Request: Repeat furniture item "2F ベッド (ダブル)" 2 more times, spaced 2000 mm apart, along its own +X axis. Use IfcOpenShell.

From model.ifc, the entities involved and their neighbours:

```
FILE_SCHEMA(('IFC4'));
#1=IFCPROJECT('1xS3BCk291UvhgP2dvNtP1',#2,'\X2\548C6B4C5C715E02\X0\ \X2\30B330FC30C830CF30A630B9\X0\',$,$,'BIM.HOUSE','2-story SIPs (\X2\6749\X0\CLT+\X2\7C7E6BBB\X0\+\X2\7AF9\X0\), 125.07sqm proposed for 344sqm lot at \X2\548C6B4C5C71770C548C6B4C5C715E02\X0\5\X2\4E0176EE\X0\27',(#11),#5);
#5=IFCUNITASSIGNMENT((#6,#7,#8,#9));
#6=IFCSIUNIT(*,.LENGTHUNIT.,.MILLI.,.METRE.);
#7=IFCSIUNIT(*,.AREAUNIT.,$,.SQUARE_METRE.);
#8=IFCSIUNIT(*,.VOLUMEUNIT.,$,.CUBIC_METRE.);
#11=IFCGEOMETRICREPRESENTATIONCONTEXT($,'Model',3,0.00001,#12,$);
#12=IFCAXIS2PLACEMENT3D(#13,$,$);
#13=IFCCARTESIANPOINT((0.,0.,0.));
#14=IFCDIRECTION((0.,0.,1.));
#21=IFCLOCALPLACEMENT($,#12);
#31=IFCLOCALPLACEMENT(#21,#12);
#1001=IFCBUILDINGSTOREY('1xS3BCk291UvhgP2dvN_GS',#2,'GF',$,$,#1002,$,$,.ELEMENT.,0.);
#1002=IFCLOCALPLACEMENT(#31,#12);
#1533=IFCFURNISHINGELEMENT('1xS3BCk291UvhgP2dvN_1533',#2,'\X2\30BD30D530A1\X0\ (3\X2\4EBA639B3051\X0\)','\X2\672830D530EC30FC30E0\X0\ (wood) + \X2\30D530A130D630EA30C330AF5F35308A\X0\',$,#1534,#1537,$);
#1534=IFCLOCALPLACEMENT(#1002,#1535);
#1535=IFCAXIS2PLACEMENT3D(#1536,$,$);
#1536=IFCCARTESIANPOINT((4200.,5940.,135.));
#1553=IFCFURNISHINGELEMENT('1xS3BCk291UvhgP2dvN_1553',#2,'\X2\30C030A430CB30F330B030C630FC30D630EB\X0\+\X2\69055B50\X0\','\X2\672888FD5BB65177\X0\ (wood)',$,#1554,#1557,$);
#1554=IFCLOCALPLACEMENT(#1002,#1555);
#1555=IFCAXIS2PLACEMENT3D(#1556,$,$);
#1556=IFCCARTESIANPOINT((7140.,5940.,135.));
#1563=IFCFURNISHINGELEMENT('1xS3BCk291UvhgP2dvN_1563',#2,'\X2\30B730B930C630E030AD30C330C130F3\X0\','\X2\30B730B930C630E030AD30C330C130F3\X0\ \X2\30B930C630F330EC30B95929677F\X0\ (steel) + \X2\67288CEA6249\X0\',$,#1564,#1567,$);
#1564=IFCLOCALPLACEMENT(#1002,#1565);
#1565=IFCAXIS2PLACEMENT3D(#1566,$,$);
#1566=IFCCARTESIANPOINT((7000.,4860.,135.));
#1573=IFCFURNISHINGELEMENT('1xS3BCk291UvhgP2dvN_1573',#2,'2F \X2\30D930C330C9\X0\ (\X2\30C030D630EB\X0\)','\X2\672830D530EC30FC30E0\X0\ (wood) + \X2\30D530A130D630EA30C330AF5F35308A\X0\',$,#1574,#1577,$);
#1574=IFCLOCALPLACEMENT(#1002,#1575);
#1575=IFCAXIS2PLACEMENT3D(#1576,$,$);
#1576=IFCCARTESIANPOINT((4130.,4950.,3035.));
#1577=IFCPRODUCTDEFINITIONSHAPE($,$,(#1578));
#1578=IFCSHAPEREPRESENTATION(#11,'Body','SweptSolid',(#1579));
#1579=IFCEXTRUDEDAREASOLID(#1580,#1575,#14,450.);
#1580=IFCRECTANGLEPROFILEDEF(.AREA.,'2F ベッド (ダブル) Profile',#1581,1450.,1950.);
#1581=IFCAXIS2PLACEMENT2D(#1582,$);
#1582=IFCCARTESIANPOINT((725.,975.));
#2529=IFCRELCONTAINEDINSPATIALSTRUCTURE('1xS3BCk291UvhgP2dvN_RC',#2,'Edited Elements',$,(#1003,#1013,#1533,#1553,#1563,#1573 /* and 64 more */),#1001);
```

```python
import ifcopenshell
import ifcopenshell.api.geometry
import ifcopenshell.api.root
import ifcopenshell.util.element
import ifcopenshell.util.placement

model = ifcopenshell.open("model.ifc")


def reuse_history(source, copy):
    """copy_class also copies each property set's owner history, people and application; keep the originals."""
    for rel in copy.IsDefinedBy:
        if rel.is_a("IfcRelDefinesByProperties") and (history := rel.RelatingPropertyDefinition.OwnerHistory):
            rel.RelatingPropertyDefinition.OwnerHistory = source.OwnerHistory
            ifcopenshell.util.element.remove_deep2(model, history)


source = model.by_guid("1xS3BCk291UvhgP2dvN_1573")
base = ifcopenshell.util.placement.get_local_placement(source.ObjectPlacement)
step = base[:3, 0] * 2000.0

for i in range(1, 3):
    copy = ifcopenshell.api.root.copy_class(model, product=source)
    copy.Representation = ifcopenshell.util.element.copy_deep(
        model, source.Representation, exclude=["IfcGeometricRepresentationContext", "IfcRepresentationMap"]
    )
    reuse_history(source, copy)
    matrix = base.copy()
    matrix[:3, 3] += i * step
    print("added at", matrix[:3, 3].round(3) + 0.0)
    ifcopenshell.api.geometry.edit_object_placement(model, product=copy, matrix=matrix, is_si=False)

model.write("model_rev.ifc")
```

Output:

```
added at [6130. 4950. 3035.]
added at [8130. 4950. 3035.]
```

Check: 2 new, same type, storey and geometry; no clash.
